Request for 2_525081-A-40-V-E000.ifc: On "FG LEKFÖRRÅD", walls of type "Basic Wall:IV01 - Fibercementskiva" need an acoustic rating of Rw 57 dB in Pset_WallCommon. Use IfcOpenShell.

First a look at what the model holds.

```python
import ifcopenshell
import ifcopenshell.util.element

model = ifcopenshell.open("2_525081-A-40-V-E000.ifc")
print(model.schema)
storey = next(s for s in model.by_type("IfcBuildingStorey") if s.Name == "FG LEKFÖRRÅD")
walls = [e for e in ifcopenshell.util.element.get_decomposition(storey) if e.is_a("IfcWall")]
seen = {}
for e in walls:
    element_type = ifcopenshell.util.element.get_type(e)
    key = (element_type.Name if element_type != e and element_type else None, ifcopenshell.util.element.get_pset(e, "Pset_WallCommon", "AcousticRating"))
    seen[key] = seen.get(key, 0) + 1
for (name, value), count in sorted(seen.items(), key=str):
    print(count, "x", name, "|", value)
```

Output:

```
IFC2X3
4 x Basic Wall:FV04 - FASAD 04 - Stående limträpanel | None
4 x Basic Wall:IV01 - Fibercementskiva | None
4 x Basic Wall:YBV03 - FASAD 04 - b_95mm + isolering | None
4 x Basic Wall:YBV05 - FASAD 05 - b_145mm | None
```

```python
import ifcopenshell
import ifcopenshell.api.pset
import ifcopenshell.util.element

model = ifcopenshell.open("2_525081-A-40-V-E000.ifc")

storey = next(s for s in model.by_type("IfcBuildingStorey") if s.Name == "FG LEKFÖRRÅD")
walls = [e for e in ifcopenshell.util.element.get_decomposition(storey) if e.is_a("IfcWall")]

count = 0
for e in walls:
    element_type = ifcopenshell.util.element.get_type(e)
    if element_type in (None, e) or element_type.Name != "Basic Wall:IV01 - Fibercementskiva":
        continue
    # add_pset returns the element's existing set when there is one.
    pset = ifcopenshell.api.pset.add_pset(model, product=e, name="Pset_WallCommon")
    ifcopenshell.api.pset.edit_pset(model, pset=pset, properties={"AcousticRating": "Rw 57 dB"})
    count += 1

print(count, "walls updated")

model.write("2_525081-A-40-V-E000_rev.ifc")
```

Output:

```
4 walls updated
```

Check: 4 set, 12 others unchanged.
